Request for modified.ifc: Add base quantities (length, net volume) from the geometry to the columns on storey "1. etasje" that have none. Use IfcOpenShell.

First a look at what the model holds.

```python
import ifcopenshell
import ifcopenshell.util.element
import ifcopenshell.util.unit

model = ifcopenshell.open("modified.ifc")
print(model.schema)
for unit_type in ("LENGTHUNIT", "AREAUNIT", "VOLUMEUNIT"):
    print(unit_type, ifcopenshell.util.unit.calculate_unit_scale(model, unit_type))
storey = next(s for s in model.by_type("IfcBuildingStorey") if s.Name == "1. etasje")
columns = [e for e in ifcopenshell.util.element.get_decomposition(storey) if e.is_a("IfcColumn")]
for e in sorted(columns, key=lambda e: e.id()):
    print(e.id(), e.is_a(), e.Name, list(ifcopenshell.util.element.get_psets(e, qtos_only=True)), sep=" | ")
```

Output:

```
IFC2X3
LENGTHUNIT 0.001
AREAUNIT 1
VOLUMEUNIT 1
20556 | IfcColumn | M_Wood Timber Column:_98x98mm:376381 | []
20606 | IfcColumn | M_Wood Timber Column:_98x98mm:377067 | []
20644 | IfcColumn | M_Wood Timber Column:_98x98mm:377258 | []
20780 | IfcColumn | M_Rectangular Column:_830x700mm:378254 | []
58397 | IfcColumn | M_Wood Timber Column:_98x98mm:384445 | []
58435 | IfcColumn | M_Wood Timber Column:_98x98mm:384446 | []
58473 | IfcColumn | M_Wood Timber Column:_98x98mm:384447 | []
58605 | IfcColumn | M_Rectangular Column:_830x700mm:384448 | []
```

```python
import ifcopenshell
import ifcopenshell.api.pset
import ifcopenshell.geom
import ifcopenshell.util.element
import ifcopenshell.util.shape
import ifcopenshell.util.unit

model = ifcopenshell.open("modified.ifc")
unit_scale = ifcopenshell.util.unit.calculate_unit_scale(model)
volume_scale = ifcopenshell.util.unit.calculate_unit_scale(model, "VOLUMEUNIT")
settings = ifcopenshell.geom.settings()

storey = next(s for s in model.by_type("IfcBuildingStorey") if s.Name == "1. etasje")
columns = [e for e in ifcopenshell.util.element.get_decomposition(storey) if e.is_a("IfcColumn")]

for e in sorted(columns, key=lambda e: e.id()):
    if ifcopenshell.util.element.get_psets(e, qtos_only=True, should_inherit=False):
        continue
    # Geometry comes back in metres, in the element's own axes.
    shape = ifcopenshell.geom.create_shape(settings, e)
    values = {
        "Length": ifcopenshell.util.shape.get_z(shape.geometry) / unit_scale,
        "NetVolume": ifcopenshell.util.shape.get_volume(shape.geometry) / volume_scale,
    }
    qto = ifcopenshell.api.pset.add_qto(model, product=e, name="BaseQuantities")
    ifcopenshell.api.pset.edit_qto(model, qto=qto, properties=values)
    print(e.id(), {k: round(v, 3) for k, v in values.items()})

model.write("modified_edited.ifc")
```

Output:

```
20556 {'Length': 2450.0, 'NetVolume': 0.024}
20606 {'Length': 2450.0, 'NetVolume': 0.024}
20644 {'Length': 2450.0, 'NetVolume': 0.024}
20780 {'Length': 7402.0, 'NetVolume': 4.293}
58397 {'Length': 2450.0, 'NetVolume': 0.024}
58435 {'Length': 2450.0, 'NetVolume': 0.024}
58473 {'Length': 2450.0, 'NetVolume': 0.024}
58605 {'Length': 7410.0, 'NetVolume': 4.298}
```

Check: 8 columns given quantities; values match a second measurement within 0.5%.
